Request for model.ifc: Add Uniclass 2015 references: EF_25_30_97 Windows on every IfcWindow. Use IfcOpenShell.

First a look at what the model holds.

```python
import ifcopenshell

model = ifcopenshell.open("model.ifc")
print(model.schema)
print("classifications:", [c.Name for c in model.by_type("IfcClassification")])
for ifc_class in ("IfcDoor", "IfcRoof", "IfcStair", "IfcWall", "IfcWindow"):
    print(ifc_class, len(model.by_type(ifc_class)))
```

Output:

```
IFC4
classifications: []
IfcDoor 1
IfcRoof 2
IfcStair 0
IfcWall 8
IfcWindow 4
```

```python
import ifcopenshell
import ifcopenshell.api.classification

model = ifcopenshell.open("model.ifc")

system = ifcopenshell.api.classification.add_classification(model, classification="Uniclass 2015")

codes = {
    "IfcWindow": ("EF_25_30_97", "Windows"),
}
for ifc_class, (code, name) in codes.items():
    products = model.by_type(ifc_class)
    ifcopenshell.api.classification.add_reference(
        model, products=products, classification=system, identification=code, name=name
    )
    print(code, len(products))

model.write("model-out.ifc")
```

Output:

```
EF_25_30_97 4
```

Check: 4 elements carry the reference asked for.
